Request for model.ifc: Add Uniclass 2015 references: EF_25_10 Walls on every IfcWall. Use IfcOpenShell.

First a look at what the model holds.

```python
import ifcopenshell

model = ifcopenshell.open("model.ifc")
print(model.schema)
print("classifications:", [c.Name for c in model.by_type("IfcClassification")])
for ifc_class in ("IfcDoor", "IfcRoof", "IfcStair", "IfcWall", "IfcWindow"):
    print(ifc_class, len(model.by_type(ifc_class)))
```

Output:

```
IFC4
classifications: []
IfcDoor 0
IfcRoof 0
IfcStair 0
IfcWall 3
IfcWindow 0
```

```python
import ifcopenshell
import ifcopenshell.api.classification

model = ifcopenshell.open("model.ifc")

system = ifcopenshell.api.classification.add_classification(model, classification="Uniclass 2015")

codes = {
    "IfcWall": ("EF_25_10", "Walls"),
}
for ifc_class, (code, name) in codes.items():
    products = model.by_type(ifc_class)
    ifcopenshell.api.classification.add_reference(
        model, products=products, classification=system, identification=code, name=name
    )
    print(code, len(products))

model.write("model_edited.ifc")
```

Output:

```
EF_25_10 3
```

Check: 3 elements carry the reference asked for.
